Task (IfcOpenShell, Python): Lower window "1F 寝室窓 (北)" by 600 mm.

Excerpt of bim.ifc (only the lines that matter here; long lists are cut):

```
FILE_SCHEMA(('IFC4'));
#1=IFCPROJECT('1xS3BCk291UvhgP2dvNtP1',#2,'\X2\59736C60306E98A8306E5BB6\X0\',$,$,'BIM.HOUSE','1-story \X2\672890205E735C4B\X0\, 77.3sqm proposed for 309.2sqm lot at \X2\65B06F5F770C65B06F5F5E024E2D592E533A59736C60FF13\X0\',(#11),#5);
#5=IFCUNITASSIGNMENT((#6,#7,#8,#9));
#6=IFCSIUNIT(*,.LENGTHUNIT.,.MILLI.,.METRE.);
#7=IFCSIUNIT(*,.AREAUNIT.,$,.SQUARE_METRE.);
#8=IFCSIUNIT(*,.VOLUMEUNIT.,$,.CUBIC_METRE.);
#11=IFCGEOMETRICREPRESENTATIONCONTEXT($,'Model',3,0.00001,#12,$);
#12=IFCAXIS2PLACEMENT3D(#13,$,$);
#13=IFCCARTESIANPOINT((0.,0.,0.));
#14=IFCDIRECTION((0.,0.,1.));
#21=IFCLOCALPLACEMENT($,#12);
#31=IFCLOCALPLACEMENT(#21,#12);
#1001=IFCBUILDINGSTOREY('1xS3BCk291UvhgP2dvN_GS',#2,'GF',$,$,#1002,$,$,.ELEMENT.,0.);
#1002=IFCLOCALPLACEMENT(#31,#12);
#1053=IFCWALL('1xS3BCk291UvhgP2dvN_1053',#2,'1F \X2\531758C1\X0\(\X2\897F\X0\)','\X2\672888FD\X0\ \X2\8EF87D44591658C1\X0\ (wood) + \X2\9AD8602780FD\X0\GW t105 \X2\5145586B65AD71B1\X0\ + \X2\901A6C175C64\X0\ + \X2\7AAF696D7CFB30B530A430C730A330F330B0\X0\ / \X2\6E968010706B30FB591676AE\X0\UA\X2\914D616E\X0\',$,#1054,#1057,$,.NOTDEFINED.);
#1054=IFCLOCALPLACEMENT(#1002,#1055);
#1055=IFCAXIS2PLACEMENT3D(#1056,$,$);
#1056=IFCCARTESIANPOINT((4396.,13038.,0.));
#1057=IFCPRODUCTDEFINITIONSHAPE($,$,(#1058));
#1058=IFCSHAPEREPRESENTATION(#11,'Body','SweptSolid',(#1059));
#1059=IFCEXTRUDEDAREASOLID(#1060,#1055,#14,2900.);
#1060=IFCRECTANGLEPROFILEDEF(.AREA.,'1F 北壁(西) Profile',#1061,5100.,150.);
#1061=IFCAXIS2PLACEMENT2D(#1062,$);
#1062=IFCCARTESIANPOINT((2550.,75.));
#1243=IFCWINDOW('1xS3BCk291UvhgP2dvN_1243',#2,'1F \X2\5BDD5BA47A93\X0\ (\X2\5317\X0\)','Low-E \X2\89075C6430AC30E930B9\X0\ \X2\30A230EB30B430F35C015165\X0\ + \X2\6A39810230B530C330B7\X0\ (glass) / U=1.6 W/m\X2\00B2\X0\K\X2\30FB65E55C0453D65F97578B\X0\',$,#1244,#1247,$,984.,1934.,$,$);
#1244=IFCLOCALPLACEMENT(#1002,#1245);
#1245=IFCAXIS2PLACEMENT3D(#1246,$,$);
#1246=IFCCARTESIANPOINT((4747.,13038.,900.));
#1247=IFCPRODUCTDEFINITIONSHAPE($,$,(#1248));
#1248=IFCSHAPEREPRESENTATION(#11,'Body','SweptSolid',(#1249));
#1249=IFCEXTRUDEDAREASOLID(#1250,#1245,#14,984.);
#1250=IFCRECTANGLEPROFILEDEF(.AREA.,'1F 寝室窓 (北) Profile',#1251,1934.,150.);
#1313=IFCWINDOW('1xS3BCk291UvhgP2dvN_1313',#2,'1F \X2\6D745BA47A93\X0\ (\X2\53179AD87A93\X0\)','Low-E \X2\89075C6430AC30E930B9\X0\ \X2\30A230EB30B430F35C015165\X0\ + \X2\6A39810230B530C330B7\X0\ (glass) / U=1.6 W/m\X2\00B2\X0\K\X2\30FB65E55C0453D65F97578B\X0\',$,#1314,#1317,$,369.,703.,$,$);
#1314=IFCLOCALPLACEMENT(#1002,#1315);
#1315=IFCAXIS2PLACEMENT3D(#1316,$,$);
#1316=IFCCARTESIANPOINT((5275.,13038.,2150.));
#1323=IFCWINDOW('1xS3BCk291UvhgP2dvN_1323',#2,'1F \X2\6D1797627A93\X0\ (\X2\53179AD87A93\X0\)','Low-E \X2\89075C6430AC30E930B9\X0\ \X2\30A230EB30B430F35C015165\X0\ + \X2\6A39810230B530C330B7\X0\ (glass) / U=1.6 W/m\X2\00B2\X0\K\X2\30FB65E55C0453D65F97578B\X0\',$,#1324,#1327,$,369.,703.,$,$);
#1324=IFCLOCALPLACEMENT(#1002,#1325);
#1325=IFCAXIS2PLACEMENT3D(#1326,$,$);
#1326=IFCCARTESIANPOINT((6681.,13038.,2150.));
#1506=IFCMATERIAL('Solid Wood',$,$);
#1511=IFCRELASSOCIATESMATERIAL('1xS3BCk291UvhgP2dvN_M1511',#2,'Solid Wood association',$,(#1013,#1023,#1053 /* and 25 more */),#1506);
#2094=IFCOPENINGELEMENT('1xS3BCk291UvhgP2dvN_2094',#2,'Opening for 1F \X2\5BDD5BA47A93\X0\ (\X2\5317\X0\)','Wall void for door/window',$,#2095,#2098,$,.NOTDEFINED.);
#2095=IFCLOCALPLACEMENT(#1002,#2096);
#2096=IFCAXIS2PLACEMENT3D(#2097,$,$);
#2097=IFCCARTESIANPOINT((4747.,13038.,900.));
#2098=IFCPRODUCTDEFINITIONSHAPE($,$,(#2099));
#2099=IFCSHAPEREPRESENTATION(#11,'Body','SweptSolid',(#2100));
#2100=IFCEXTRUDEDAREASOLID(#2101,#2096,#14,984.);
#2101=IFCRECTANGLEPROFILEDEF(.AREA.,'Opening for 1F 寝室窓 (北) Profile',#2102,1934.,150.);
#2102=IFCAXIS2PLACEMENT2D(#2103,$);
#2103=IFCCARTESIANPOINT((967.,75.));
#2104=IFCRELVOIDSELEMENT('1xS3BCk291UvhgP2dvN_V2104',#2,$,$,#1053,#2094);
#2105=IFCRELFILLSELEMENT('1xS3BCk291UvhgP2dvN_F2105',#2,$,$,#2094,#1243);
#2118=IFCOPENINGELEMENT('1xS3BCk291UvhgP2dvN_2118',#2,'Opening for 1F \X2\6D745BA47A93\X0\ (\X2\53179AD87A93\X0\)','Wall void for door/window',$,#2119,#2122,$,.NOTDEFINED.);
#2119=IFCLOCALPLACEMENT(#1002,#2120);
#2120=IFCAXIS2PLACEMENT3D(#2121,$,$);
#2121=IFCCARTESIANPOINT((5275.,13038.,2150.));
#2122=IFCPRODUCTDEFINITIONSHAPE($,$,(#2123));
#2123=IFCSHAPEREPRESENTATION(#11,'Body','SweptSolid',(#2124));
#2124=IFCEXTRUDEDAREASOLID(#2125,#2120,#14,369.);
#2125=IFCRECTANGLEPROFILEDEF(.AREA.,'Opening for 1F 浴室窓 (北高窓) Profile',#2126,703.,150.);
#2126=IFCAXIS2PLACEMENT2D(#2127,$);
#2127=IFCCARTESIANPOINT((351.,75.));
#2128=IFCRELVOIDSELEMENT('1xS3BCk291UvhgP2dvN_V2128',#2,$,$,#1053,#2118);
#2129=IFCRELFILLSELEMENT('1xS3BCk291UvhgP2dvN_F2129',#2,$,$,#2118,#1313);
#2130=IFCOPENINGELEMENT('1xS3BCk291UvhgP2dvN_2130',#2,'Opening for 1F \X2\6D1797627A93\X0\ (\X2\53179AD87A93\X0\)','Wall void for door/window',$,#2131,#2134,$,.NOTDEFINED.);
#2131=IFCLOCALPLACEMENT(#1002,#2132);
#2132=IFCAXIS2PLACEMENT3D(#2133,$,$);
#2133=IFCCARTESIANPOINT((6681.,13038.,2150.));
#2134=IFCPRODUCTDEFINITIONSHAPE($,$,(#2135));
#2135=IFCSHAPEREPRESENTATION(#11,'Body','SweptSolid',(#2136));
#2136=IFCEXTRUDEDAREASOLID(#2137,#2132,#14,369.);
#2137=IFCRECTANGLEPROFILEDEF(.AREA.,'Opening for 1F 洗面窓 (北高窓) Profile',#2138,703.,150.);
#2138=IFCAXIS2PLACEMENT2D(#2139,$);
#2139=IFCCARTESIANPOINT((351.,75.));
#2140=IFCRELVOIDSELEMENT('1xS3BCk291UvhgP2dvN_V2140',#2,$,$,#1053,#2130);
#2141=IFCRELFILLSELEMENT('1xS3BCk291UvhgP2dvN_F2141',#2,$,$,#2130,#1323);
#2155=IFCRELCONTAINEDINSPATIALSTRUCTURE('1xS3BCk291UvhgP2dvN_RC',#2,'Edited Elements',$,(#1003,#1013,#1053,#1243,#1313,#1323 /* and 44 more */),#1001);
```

```python
import numpy as np
import ifcopenshell
import ifcopenshell.api.geometry
import ifcopenshell.util.placement
import ifcopenshell.util.unit

model = ifcopenshell.open("bim.ifc")
unit_scale = ifcopenshell.util.unit.calculate_unit_scale(model)

window = model.by_guid("1xS3BCk291UvhgP2dvN_1243")
opening = window.FillsVoids[0].RelatingOpeningElement
dz = -600.0

shift = np.array([0.0, 0.0, dz])
# The window is not placed relative to its opening, so move both.
for product in (opening, window):
    matrix = ifcopenshell.util.placement.get_local_placement(product.ObjectPlacement)
    matrix[:3, 3] += shift
    ifcopenshell.api.geometry.edit_object_placement(model, product=product, matrix=matrix, is_si=False)

print(f"moved by {dz * unit_scale:+.3f} m")

model.write("bim_rev.ifc")
```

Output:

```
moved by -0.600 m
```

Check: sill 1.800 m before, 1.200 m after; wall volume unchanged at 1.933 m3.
